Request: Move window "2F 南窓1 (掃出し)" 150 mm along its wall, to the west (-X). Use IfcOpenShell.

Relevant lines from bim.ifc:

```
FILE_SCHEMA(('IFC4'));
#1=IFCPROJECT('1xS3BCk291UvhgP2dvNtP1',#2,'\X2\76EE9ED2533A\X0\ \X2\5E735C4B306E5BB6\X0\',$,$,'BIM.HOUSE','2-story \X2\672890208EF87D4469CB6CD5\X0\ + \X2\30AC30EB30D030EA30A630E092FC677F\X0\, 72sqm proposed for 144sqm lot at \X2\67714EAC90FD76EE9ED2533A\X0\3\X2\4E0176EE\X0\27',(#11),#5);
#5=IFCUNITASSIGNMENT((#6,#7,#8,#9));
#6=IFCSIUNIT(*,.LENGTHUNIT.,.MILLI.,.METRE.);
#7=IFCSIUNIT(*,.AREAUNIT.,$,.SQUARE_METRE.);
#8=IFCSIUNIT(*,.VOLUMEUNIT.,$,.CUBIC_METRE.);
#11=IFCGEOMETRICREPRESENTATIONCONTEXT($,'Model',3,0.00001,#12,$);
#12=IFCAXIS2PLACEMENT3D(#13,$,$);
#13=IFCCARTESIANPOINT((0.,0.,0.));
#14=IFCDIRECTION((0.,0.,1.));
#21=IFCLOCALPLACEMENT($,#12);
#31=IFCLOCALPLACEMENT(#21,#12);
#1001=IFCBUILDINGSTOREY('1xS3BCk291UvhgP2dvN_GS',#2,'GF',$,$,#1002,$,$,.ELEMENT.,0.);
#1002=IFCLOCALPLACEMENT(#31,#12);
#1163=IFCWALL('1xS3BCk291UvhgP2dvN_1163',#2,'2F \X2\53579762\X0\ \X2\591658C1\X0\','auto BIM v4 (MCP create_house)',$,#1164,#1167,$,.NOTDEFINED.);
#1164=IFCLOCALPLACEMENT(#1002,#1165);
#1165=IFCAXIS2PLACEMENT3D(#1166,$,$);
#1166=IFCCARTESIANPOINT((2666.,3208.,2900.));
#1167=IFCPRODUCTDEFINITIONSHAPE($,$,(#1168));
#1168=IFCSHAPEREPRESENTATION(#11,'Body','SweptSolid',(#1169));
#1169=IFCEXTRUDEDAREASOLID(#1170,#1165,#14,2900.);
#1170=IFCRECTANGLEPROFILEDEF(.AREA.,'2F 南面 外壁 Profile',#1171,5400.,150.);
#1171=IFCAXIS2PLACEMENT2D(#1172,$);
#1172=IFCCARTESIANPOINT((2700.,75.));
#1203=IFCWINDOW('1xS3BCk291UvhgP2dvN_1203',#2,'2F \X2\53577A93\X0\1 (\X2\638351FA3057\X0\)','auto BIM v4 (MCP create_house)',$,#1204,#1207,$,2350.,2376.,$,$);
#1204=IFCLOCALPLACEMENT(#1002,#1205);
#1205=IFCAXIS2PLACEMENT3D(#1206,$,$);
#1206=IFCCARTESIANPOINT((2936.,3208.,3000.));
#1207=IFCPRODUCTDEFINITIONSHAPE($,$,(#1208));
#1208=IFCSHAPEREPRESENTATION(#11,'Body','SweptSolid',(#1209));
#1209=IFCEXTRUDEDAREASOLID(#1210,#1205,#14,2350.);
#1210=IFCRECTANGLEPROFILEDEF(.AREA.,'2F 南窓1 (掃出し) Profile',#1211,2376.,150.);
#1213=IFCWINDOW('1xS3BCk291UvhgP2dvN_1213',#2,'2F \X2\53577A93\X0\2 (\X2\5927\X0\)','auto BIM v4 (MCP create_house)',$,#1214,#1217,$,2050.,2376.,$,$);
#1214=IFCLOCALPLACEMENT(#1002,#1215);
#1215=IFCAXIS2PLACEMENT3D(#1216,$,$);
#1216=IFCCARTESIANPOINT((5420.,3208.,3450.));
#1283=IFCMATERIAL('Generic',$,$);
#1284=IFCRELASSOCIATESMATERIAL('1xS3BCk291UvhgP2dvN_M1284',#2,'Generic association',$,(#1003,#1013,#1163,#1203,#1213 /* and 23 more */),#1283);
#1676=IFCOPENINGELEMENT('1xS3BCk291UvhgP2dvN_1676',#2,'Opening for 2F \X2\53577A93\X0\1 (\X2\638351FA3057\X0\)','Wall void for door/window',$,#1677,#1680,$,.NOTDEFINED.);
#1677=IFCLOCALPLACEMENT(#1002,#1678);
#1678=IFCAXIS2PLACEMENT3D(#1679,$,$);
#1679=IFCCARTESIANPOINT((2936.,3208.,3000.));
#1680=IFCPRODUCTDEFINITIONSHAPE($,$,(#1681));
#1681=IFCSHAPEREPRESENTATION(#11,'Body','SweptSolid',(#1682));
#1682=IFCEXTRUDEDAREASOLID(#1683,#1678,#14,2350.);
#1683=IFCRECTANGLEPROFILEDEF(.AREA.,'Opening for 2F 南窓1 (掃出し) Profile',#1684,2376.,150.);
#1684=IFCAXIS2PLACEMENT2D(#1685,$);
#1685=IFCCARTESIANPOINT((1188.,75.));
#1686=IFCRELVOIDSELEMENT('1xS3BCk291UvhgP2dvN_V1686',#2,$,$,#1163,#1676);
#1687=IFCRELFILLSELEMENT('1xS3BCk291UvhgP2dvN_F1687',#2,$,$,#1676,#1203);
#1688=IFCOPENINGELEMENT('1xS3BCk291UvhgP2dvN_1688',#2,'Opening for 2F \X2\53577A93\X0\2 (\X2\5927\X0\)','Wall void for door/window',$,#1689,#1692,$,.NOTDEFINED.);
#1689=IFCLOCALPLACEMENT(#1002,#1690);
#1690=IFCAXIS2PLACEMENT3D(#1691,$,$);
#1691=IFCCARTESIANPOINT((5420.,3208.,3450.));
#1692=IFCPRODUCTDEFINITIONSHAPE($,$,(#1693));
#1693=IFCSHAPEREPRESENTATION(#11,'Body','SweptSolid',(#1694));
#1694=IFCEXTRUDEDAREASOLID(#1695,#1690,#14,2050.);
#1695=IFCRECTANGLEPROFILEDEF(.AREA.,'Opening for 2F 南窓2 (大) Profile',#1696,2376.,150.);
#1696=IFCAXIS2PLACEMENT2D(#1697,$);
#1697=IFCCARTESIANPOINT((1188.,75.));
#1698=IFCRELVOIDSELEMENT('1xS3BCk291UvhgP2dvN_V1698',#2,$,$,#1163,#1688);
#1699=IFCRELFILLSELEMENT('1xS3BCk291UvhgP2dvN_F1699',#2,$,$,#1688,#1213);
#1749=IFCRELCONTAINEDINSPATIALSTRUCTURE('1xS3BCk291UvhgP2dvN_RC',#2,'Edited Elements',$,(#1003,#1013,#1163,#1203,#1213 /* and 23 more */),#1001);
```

```python
import ifcopenshell
import ifcopenshell.api.geometry
import ifcopenshell.util.placement

model = ifcopenshell.open("bim.ifc")

window = model.by_guid("1xS3BCk291UvhgP2dvN_1203")
opening = window.FillsVoids[0].RelatingOpeningElement
wall = opening.VoidsElements[0].RelatingBuildingElement

wall_matrix = ifcopenshell.util.placement.get_local_placement(wall.ObjectPlacement)
shift = wall_matrix[:3, 0] * -150.0
before = ifcopenshell.util.placement.get_local_placement(window.ObjectPlacement)[:3, 3].copy()

# The window is not placed relative to its opening, so move both.
for product in (opening, window):
    matrix = ifcopenshell.util.placement.get_local_placement(product.ObjectPlacement)
    matrix[:3, 3] += shift
    ifcopenshell.api.geometry.edit_object_placement(model, product=product, matrix=matrix, is_si=False)

after = ifcopenshell.util.placement.get_local_placement(window.ObjectPlacement)[:3, 3]
print("window moved by", (after - before).round(3) + 0.0)

model.write("bim_v2.ifc")
```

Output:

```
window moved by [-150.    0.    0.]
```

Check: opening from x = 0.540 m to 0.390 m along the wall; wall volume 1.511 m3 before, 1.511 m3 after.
